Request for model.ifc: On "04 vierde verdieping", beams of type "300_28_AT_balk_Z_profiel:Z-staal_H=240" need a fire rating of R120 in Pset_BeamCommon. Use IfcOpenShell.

First a look at what the model holds.

```python
import ifcopenshell
import ifcopenshell.util.element

model = ifcopenshell.open("model.ifc")
print(model.schema)
storey = next(s for s in model.by_type("IfcBuildingStorey") if s.Name == "04 vierde verdieping")
beams = [e for e in ifcopenshell.util.element.get_decomposition(storey) if e.is_a("IfcBeam")]
seen = {}
for e in beams:
    element_type = ifcopenshell.util.element.get_type(e)
    key = (element_type.Name if element_type != e and element_type else None, ifcopenshell.util.element.get_pset(e, "Pset_BeamCommon", "FireRating"))
    seen[key] = seen.get(key, 0) + 1
for (name, value), count in sorted(seen.items(), key=str):
    print(count, "x", name, "|", value)
```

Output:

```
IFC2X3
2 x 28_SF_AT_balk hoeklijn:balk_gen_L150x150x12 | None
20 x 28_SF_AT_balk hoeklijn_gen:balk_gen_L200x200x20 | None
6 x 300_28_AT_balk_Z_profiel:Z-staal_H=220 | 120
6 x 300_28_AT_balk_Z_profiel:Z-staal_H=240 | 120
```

```python
import ifcopenshell
import ifcopenshell.api.pset
import ifcopenshell.util.element

model = ifcopenshell.open("model.ifc")

storey = next(s for s in model.by_type("IfcBuildingStorey") if s.Name == "04 vierde verdieping")
beams = [e for e in ifcopenshell.util.element.get_decomposition(storey) if e.is_a("IfcBeam")]

count = 0
for e in beams:
    element_type = ifcopenshell.util.element.get_type(e)
    if element_type in (None, e) or element_type.Name != "300_28_AT_balk_Z_profiel:Z-staal_H=240":
        continue
    # add_pset returns the element's existing set when there is one.
    pset = ifcopenshell.api.pset.add_pset(model, product=e, name="Pset_BeamCommon")
    ifcopenshell.api.pset.edit_pset(model, pset=pset, properties={"FireRating": "R120"})
    count += 1

print(count, "beams updated")

model.write("model-out.ifc")
```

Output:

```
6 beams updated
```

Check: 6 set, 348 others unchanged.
